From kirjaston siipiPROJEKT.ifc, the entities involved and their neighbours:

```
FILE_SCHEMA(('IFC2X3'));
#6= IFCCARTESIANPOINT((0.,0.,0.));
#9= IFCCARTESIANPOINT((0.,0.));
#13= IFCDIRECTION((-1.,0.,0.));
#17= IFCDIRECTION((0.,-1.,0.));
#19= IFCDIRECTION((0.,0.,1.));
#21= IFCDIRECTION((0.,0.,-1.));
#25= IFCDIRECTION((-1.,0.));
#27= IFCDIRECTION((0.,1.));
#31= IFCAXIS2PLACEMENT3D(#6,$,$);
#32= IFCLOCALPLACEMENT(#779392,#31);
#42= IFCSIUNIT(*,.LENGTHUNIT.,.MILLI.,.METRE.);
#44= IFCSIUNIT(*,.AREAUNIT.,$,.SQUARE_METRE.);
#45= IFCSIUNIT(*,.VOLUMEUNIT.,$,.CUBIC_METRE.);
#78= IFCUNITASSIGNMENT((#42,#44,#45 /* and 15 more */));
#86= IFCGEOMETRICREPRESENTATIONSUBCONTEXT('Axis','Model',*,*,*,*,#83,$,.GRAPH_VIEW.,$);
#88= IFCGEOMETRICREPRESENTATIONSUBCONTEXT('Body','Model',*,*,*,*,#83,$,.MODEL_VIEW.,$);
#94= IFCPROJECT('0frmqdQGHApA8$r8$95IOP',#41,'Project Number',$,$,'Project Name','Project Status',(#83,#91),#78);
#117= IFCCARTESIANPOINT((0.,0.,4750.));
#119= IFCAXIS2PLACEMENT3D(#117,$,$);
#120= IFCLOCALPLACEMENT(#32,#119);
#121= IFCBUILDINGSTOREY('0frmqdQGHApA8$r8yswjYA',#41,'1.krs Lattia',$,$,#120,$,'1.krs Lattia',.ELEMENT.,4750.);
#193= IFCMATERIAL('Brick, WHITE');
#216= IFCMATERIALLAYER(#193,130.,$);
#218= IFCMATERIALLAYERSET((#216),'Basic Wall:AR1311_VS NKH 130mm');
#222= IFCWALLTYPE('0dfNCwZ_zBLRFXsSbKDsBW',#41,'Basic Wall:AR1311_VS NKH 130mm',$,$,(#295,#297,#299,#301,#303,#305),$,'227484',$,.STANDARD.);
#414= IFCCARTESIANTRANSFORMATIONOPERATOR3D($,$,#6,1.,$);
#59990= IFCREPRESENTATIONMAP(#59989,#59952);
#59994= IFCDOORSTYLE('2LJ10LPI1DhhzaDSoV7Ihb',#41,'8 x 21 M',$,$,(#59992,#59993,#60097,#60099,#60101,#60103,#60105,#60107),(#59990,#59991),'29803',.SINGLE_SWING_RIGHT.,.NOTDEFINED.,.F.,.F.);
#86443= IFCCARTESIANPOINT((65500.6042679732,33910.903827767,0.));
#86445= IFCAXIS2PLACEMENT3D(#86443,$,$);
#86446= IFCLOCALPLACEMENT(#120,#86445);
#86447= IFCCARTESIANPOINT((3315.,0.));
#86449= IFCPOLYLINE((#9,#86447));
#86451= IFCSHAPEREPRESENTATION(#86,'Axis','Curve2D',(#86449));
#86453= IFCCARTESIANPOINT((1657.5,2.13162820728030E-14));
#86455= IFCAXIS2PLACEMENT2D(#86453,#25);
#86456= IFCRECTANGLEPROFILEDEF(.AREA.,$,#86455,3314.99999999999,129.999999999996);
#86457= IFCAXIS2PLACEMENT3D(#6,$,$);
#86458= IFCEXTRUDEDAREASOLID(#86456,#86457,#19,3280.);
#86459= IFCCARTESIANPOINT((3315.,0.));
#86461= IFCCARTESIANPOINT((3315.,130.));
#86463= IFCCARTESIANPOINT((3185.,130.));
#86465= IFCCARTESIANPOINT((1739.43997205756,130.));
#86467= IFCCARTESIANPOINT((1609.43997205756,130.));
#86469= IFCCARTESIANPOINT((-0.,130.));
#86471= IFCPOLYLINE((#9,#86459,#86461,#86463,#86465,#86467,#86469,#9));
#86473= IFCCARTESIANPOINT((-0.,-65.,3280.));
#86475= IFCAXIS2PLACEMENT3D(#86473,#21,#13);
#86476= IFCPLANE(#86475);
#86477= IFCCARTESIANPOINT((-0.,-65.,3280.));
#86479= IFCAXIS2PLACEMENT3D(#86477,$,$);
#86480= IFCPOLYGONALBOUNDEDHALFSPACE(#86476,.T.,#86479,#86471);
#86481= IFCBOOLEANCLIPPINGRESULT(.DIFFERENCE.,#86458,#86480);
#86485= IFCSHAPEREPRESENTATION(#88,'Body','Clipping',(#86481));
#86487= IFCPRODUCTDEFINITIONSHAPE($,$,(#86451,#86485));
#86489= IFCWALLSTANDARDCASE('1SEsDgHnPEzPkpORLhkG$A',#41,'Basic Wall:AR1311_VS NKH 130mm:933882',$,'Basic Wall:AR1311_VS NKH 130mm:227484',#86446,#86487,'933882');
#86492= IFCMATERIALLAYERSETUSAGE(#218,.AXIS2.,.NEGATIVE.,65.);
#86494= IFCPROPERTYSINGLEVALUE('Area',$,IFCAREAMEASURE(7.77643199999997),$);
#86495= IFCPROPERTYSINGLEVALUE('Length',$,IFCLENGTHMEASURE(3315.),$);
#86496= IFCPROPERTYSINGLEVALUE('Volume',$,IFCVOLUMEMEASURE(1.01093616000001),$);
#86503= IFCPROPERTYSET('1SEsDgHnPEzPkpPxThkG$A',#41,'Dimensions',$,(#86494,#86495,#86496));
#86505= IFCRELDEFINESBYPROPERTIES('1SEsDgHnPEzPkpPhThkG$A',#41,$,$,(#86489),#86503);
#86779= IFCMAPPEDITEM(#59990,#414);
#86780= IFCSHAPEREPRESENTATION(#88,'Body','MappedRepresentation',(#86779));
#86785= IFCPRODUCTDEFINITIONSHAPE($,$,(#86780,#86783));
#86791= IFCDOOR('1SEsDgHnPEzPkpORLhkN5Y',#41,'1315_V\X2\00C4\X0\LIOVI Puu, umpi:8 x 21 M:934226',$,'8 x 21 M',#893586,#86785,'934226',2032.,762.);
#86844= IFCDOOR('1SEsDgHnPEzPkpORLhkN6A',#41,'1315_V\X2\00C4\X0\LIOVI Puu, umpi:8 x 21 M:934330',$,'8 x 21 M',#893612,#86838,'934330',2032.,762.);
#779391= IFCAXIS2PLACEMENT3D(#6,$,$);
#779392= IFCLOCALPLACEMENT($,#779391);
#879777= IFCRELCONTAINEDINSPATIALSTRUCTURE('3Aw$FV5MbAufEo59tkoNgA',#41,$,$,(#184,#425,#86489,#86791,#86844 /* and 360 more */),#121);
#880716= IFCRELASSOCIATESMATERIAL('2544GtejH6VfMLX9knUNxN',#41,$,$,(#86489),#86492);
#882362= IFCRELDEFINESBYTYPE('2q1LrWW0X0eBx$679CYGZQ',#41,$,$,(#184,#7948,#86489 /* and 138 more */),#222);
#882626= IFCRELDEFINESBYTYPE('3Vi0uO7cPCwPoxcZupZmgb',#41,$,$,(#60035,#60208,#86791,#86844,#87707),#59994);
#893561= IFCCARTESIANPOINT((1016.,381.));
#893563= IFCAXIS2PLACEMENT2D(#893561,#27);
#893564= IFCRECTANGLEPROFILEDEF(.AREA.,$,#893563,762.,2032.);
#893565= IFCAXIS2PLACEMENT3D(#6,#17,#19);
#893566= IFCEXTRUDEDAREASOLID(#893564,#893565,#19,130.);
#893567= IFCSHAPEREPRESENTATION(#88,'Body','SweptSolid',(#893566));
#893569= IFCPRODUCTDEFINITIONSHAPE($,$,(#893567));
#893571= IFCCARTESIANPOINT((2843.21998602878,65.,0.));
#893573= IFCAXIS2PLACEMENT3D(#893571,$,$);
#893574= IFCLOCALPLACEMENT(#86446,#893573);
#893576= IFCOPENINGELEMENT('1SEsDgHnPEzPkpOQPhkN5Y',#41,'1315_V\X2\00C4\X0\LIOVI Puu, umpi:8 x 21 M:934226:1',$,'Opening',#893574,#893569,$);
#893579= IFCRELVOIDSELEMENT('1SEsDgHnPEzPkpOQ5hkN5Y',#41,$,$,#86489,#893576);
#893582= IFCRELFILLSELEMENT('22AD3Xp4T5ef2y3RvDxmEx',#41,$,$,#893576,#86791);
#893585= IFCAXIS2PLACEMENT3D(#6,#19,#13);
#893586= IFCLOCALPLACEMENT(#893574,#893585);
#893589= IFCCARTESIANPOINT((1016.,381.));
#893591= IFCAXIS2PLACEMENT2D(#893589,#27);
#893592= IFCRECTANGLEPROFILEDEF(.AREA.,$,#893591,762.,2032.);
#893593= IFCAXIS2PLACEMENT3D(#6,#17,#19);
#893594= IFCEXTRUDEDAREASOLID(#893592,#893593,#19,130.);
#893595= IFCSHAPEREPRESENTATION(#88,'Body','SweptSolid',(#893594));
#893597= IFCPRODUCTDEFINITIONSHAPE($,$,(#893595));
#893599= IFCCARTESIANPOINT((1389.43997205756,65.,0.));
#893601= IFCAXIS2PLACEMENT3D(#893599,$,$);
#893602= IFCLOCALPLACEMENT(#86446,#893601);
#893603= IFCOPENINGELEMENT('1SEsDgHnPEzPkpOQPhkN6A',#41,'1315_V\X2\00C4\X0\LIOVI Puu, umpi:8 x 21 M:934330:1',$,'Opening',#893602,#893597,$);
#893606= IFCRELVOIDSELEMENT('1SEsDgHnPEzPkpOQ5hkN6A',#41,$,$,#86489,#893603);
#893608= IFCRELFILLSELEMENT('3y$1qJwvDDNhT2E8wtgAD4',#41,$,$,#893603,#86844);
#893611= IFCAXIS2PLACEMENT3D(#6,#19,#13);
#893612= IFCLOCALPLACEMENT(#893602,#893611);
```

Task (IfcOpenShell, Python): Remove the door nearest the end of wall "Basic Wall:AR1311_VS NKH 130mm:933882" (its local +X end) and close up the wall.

```python
import ifcopenshell
import ifcopenshell.api.feature
import ifcopenshell.api.pset
import ifcopenshell.api.root
import ifcopenshell.geom
import ifcopenshell.util.element
import ifcopenshell.util.shape
import ifcopenshell.util.unit

model = ifcopenshell.open("kirjaston siipiPROJEKT.ifc")
area_scale = ifcopenshell.util.unit.calculate_unit_scale(model, "AREAUNIT")
volume_scale = ifcopenshell.util.unit.calculate_unit_scale(model, "VOLUMEUNIT")
settings = ifcopenshell.geom.settings()


def volume(element):
    """Net volume in cubic metres, openings subtracted."""
    shape = ifcopenshell.geom.create_shape(settings, element)
    return ifcopenshell.util.shape.get_volume(shape.geometry)


door = model.by_id(86791)
opening = door.FillsVoids[0].RelatingOpeningElement
wall = opening.VoidsElements[0].RelatingBuildingElement
before = volume(wall)

ifcopenshell.api.root.remove_product(model, product=door)
ifcopenshell.api.feature.remove_feature(model, feature=opening)

after = volume(wall)
thickness = 0.13  # wall thickness in metres

# Update the wall's stored quantities.
pset = model.by_id(ifcopenshell.util.element.get_pset(wall, "Dimensions", should_inherit=False)["id"])
ifcopenshell.api.pset.edit_pset(model, pset=pset, properties={
    "Area": model.create_entity("IfcAreaMeasure", after / thickness / area_scale),
    "Volume": model.create_entity("IfcVolumeMeasure", after / volume_scale),
})

print(f"wall volume {before:.3f} -> {after:.3f} m3")

model.write("kirjaston siipiPROJEKT_edited.ifc")
```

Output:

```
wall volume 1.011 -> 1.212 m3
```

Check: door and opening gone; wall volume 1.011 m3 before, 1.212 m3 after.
